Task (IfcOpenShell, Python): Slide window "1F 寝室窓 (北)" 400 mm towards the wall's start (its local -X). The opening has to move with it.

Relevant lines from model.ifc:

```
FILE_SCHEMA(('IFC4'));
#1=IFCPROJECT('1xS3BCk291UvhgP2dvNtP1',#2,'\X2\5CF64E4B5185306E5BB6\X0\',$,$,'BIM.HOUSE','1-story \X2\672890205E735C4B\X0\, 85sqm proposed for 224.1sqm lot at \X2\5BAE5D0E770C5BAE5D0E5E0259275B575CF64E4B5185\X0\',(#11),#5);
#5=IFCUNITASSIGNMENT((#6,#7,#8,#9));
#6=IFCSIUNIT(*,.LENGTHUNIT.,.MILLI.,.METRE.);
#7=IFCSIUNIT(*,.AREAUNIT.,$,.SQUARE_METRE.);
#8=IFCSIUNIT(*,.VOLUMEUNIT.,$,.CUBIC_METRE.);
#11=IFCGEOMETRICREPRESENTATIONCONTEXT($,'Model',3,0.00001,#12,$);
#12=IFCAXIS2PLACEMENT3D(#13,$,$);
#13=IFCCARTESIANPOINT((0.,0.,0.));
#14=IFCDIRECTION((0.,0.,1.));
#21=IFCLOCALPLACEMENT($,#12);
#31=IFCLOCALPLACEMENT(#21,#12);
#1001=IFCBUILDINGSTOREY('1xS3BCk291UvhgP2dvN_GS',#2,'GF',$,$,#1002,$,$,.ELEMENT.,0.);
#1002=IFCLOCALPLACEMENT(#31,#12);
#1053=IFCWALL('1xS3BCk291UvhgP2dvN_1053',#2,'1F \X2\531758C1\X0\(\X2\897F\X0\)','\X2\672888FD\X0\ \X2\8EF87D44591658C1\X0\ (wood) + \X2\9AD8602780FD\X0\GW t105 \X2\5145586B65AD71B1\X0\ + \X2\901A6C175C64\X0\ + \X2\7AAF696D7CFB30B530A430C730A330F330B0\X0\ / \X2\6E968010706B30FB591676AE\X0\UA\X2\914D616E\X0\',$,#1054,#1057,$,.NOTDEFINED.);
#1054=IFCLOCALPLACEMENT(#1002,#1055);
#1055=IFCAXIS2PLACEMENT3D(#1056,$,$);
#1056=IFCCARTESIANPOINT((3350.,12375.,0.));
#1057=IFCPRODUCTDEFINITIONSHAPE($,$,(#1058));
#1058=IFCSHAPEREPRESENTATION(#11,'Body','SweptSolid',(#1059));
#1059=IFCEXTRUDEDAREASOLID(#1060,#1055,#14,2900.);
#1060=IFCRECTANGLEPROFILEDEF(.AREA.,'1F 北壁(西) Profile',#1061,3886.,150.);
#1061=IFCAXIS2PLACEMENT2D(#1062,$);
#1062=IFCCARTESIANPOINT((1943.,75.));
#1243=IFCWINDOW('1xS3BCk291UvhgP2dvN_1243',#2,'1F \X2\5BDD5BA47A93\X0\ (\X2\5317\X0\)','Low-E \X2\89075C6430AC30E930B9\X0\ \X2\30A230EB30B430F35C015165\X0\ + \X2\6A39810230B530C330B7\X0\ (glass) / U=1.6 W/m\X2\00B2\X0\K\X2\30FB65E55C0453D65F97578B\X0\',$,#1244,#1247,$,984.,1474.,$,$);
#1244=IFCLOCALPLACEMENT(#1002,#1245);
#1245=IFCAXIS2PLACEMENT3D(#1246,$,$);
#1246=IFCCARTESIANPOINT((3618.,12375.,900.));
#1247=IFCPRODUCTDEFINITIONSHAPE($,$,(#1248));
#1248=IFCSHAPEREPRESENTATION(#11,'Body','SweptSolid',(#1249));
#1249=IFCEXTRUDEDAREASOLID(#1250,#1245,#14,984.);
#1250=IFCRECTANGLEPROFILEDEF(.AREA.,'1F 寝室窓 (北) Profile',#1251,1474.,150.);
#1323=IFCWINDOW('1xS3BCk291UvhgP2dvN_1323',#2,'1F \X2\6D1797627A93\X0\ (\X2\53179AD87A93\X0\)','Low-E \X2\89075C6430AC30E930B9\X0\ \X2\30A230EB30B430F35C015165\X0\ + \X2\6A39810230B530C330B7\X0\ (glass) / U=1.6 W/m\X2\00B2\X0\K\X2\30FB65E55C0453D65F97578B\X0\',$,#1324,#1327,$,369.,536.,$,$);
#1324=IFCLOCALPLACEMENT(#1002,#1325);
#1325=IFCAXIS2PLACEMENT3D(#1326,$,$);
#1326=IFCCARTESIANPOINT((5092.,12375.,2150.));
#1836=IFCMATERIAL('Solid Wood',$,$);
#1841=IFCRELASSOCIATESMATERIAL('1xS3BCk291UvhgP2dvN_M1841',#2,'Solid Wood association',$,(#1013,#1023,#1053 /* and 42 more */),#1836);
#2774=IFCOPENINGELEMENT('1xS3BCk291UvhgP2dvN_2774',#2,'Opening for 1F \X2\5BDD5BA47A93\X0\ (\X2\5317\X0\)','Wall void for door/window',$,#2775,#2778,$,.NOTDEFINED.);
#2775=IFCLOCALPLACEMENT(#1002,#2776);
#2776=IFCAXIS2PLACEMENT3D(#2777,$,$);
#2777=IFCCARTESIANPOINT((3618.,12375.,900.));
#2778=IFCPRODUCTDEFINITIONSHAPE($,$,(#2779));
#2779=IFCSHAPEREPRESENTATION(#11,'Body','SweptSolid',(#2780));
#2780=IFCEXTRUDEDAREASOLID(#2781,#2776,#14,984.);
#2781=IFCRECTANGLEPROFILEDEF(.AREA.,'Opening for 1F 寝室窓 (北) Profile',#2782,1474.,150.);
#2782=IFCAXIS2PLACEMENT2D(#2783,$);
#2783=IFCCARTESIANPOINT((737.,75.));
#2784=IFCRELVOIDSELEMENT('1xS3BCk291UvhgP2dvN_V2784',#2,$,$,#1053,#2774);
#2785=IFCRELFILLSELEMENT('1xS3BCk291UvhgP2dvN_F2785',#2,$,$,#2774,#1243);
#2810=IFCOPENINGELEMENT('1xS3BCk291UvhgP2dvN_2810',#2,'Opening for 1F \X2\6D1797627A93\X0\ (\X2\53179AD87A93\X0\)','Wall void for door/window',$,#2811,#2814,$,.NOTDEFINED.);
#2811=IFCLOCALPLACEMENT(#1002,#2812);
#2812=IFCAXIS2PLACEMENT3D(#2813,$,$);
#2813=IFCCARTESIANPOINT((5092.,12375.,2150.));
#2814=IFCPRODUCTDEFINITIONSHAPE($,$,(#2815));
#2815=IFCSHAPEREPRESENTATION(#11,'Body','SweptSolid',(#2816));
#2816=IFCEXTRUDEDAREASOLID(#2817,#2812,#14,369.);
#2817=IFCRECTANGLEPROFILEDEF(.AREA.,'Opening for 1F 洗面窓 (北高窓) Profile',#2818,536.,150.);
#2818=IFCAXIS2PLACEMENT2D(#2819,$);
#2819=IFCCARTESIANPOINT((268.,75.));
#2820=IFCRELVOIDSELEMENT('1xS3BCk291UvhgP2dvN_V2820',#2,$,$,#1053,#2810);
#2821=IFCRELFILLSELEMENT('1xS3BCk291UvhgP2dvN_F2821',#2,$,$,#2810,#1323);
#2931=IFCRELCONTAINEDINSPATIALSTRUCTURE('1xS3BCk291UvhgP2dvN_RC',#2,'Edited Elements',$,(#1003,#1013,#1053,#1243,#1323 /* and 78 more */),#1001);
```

```python
import ifcopenshell
import ifcopenshell.api.geometry
import ifcopenshell.util.placement
import ifcopenshell.util.unit

model = ifcopenshell.open("model.ifc")
unit_scale = ifcopenshell.util.unit.calculate_unit_scale(model)

window = model.by_id(1243)
opening = window.FillsVoids[0].RelatingOpeningElement
wall = opening.VoidsElements[0].RelatingBuildingElement

wall_matrix = ifcopenshell.util.placement.get_local_placement(wall.ObjectPlacement)
shift = wall_matrix[:3, 0] * -0.4 / unit_scale
before = ifcopenshell.util.placement.get_local_placement(window.ObjectPlacement)[:3, 3].copy()

# The window is not placed relative to its opening, so move both.
for product in (opening, window):
    matrix = ifcopenshell.util.placement.get_local_placement(product.ObjectPlacement)
    matrix[:3, 3] += shift
    ifcopenshell.api.geometry.edit_object_placement(model, product=product, matrix=matrix, is_si=False)

after = ifcopenshell.util.placement.get_local_placement(window.ObjectPlacement)[:3, 3]
print("window moved by", (after - before).round(3) + 0.0)

model.write("model_rev.ifc")
```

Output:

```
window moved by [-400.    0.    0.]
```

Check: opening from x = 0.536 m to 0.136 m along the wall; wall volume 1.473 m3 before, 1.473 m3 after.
